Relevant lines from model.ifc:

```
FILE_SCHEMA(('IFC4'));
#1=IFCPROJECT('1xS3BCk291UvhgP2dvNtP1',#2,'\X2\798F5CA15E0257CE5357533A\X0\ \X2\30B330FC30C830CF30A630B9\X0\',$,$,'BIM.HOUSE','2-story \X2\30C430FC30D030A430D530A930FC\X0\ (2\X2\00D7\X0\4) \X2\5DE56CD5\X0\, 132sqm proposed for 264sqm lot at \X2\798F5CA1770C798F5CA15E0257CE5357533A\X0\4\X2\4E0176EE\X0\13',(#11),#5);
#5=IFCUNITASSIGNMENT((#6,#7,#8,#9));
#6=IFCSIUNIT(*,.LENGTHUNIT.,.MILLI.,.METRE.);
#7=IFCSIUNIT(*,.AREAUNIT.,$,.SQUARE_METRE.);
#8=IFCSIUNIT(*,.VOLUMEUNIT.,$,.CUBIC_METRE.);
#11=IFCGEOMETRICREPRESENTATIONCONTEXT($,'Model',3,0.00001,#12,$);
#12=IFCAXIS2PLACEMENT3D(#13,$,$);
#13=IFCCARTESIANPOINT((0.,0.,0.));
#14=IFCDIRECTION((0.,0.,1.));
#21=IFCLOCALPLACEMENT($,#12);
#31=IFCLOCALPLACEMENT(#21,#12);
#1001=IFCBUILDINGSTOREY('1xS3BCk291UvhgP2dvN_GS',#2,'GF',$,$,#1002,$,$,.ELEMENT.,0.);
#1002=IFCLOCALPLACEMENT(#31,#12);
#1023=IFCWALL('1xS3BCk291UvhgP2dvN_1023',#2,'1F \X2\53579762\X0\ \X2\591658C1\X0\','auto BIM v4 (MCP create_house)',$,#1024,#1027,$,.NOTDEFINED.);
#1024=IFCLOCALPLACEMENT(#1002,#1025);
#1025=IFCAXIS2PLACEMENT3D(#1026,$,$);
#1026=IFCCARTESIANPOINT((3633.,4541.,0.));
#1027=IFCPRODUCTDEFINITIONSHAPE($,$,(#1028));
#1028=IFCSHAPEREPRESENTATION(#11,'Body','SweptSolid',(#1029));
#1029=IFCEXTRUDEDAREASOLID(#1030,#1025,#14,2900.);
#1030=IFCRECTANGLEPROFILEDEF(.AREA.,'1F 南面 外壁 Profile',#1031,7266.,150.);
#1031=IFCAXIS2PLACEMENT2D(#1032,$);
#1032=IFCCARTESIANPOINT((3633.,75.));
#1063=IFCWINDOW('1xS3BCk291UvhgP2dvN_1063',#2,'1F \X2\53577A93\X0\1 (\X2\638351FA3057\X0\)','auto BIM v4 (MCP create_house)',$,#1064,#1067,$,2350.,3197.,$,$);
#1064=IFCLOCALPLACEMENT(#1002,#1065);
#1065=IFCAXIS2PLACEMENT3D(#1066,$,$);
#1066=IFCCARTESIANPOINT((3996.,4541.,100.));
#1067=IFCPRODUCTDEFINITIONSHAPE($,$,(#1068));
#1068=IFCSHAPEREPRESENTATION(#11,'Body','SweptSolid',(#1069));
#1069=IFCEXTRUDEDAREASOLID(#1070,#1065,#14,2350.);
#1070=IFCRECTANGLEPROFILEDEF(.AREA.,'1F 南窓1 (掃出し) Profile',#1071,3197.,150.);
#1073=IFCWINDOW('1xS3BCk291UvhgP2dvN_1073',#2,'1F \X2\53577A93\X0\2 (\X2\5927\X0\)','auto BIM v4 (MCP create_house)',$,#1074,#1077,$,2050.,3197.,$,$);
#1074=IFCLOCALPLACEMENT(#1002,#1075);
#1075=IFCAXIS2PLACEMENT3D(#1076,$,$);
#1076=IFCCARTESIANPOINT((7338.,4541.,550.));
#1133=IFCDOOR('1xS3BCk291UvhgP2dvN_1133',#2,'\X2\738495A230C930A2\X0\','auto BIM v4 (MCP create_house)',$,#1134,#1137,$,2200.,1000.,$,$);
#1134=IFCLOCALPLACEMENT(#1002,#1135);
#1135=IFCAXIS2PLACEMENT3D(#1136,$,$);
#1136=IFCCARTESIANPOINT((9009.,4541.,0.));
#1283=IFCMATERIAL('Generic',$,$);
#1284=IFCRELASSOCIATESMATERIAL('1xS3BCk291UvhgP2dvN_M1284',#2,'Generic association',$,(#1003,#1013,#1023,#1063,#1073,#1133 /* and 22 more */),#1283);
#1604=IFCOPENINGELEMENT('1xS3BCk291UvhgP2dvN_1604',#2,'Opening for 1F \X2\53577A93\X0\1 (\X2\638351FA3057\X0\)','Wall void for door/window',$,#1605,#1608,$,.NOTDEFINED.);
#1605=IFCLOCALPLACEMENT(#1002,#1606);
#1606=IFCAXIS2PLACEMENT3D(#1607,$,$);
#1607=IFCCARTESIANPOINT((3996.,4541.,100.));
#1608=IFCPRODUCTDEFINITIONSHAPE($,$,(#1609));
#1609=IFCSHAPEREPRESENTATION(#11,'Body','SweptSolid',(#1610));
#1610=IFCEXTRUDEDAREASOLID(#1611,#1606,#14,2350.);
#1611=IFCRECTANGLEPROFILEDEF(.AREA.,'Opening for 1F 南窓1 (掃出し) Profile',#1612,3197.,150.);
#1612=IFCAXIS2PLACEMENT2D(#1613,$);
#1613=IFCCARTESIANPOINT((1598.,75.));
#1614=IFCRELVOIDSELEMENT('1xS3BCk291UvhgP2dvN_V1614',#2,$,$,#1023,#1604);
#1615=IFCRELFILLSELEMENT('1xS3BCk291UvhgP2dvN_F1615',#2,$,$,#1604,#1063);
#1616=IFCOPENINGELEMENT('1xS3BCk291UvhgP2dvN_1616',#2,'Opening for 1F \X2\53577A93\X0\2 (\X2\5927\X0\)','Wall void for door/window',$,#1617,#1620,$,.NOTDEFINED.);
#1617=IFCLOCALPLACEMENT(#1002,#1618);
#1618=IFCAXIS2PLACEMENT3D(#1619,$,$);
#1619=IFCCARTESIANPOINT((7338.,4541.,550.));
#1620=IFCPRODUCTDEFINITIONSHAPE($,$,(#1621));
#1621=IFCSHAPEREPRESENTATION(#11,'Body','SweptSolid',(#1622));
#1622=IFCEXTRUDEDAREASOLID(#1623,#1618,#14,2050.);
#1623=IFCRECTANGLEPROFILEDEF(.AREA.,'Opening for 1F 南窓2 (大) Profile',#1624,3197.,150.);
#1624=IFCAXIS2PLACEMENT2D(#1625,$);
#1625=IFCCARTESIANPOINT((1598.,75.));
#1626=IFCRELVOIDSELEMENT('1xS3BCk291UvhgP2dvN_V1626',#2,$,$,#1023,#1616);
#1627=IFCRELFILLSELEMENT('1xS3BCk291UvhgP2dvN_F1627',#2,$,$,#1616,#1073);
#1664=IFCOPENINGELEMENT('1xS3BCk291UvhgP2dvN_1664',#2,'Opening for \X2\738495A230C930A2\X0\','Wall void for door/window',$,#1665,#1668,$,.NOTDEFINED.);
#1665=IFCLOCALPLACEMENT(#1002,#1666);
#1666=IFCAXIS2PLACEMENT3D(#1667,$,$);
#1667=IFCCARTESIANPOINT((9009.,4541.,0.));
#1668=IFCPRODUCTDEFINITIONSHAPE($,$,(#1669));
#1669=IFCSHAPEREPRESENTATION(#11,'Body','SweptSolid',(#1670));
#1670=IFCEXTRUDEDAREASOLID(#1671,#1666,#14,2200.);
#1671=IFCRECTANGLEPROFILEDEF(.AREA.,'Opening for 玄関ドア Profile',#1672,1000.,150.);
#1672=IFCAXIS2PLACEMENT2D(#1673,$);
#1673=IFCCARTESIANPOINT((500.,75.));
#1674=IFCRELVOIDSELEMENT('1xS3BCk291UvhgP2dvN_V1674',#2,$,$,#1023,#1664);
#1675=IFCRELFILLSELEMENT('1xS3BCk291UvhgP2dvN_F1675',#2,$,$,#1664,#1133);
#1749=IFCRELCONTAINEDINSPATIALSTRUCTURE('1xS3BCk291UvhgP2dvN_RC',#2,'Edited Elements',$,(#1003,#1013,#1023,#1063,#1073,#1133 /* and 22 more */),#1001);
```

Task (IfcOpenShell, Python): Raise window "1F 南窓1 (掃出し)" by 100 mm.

```python
import numpy as np
import ifcopenshell
import ifcopenshell.api.geometry
import ifcopenshell.util.placement
import ifcopenshell.util.unit

model = ifcopenshell.open("model.ifc")
unit_scale = ifcopenshell.util.unit.calculate_unit_scale(model)

window = model.by_id(1063)
opening = window.FillsVoids[0].RelatingOpeningElement
dz = 100.0

shift = np.array([0.0, 0.0, dz])
# The window is not placed relative to its opening, so move both.
for product in (opening, window):
    matrix = ifcopenshell.util.placement.get_local_placement(product.ObjectPlacement)
    matrix[:3, 3] += shift
    ifcopenshell.api.geometry.edit_object_placement(model, product=product, matrix=matrix, is_si=False)

print(f"moved by {dz * unit_scale:+.3f} m")

model.write("model_edited.ifc")
```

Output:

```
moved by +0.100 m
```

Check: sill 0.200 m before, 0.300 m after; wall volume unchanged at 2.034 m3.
